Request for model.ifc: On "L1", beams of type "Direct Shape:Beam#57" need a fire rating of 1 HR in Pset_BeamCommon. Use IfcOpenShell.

First a look at what the model holds.

```python
import ifcopenshell
import ifcopenshell.util.element

model = ifcopenshell.open("model.ifc")
print(model.schema)
storey = next(s for s in model.by_type("IfcBuildingStorey") if s.Name == "L1")
beams = [e for e in ifcopenshell.util.element.get_decomposition(storey) if e.is_a("IfcBeam")]
seen = {}
for e in beams:
    element_type = ifcopenshell.util.element.get_type(e)
    key = (element_type.Name if element_type != e and element_type else None, ifcopenshell.util.element.get_pset(e, "Pset_BeamCommon", "FireRating"))
    seen[key] = seen.get(key, 0) + 1
for (name, value), count in sorted(seen.items(), key=str):
    print(count, "x", name, "|", value)
```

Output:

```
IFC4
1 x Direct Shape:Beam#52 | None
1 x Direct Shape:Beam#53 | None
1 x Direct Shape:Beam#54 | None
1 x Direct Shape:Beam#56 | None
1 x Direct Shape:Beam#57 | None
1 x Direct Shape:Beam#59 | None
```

```python
import ifcopenshell
import ifcopenshell.api.pset
import ifcopenshell.util.element

model = ifcopenshell.open("model.ifc")

storey = next(s for s in model.by_type("IfcBuildingStorey") if s.Name == "L1")
beams = [e for e in ifcopenshell.util.element.get_decomposition(storey) if e.is_a("IfcBeam")]

count = 0
for e in beams:
    element_type = ifcopenshell.util.element.get_type(e)
    if element_type in (None, e) or element_type.Name != "Direct Shape:Beam#57":
        continue
    # add_pset returns the element's existing set when there is one.
    pset = ifcopenshell.api.pset.add_pset(model, product=e, name="Pset_BeamCommon")
    ifcopenshell.api.pset.edit_pset(model, pset=pset, properties={"FireRating": "1 HR"})
    count += 1

print(count, "beams updated")

model.write("model_v2.ifc")
```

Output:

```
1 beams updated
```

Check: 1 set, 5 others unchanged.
